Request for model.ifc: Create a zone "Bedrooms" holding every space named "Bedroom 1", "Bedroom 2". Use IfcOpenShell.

First a look at what the model holds.

```python
import ifcopenshell

model = ifcopenshell.open("model.ifc")
print(model.schema)
seen = {}
for space in model.by_type("IfcSpace"):
    seen[space.LongName] = seen.get(space.LongName, 0) + 1
for name, count in sorted(seen.items(), key=str):
    print(count, "x", name)
print("zones:", [z.Name for z in model.by_type("IfcZone")][:20])
```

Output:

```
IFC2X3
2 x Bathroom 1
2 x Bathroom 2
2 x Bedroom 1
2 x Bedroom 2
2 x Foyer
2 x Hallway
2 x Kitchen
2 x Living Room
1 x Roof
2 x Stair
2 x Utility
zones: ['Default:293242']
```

```python
import ifcopenshell
import ifcopenshell.api.group
import ifcopenshell.api.root

model = ifcopenshell.open("model.ifc")

names = {"Bedroom 1", "Bedroom 2"}
spaces = [s for s in model.by_type("IfcSpace") if s.LongName in names]

zone = ifcopenshell.api.root.create_entity(model, ifc_class="IfcZone", name="Bedrooms")
ifcopenshell.api.group.assign_group(model, products=spaces, group=zone)
print(len(spaces), "spaces in", zone.Name)

model.write("model_updated.ifc")
```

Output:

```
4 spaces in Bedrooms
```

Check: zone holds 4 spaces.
